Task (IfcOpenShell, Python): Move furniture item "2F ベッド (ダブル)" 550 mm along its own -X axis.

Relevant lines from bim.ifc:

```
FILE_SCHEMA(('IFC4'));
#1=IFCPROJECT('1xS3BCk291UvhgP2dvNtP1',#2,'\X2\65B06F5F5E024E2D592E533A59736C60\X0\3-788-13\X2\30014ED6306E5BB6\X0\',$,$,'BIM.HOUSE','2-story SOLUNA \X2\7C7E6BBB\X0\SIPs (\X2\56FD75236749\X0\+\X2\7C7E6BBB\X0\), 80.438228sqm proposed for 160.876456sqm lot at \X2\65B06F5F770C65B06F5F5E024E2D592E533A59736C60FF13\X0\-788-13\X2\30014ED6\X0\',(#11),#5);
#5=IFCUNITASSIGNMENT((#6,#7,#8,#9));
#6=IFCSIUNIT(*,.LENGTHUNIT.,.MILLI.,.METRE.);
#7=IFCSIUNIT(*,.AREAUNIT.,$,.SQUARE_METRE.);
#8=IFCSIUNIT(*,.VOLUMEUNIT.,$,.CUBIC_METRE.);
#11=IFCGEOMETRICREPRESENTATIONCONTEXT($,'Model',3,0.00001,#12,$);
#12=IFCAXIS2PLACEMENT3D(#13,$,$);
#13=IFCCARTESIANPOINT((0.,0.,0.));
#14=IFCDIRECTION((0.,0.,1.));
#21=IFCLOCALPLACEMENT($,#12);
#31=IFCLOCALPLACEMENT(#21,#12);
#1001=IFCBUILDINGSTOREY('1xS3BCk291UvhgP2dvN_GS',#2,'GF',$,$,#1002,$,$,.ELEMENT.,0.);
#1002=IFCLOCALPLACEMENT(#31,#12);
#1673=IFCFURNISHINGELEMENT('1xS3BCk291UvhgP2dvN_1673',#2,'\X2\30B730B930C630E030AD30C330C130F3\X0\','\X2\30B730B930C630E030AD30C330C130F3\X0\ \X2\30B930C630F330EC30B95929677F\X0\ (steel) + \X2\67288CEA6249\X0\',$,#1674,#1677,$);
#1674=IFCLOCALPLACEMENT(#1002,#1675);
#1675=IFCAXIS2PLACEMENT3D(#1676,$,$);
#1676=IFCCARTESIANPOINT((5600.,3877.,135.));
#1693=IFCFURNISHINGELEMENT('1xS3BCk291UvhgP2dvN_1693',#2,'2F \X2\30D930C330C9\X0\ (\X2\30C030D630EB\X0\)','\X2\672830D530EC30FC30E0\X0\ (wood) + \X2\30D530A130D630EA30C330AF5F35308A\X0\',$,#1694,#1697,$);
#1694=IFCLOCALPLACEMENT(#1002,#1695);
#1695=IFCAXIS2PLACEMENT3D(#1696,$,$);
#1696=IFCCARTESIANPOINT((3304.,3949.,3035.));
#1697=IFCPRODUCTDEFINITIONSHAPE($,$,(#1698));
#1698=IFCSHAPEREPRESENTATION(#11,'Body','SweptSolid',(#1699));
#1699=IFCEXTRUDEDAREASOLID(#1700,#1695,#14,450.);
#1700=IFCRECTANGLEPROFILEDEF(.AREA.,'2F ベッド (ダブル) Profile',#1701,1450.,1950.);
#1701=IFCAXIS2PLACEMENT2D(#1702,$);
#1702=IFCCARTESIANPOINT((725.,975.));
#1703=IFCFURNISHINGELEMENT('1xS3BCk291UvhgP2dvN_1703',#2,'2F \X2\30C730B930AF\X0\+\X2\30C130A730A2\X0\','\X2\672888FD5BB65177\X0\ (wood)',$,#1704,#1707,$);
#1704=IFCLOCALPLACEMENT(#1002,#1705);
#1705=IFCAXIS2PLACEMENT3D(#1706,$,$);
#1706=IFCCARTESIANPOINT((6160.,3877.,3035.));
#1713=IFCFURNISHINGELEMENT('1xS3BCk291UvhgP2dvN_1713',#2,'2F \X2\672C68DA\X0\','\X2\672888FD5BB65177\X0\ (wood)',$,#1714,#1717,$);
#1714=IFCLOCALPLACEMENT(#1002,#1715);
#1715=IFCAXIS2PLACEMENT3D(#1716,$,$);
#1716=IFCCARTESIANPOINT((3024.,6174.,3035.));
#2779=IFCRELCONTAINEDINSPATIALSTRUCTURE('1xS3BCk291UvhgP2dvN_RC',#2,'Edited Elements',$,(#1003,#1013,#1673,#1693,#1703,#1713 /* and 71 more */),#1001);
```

```python
import ifcopenshell
import ifcopenshell.api.geometry
import ifcopenshell.util.placement

model = ifcopenshell.open("bim.ifc")

item = model.by_guid("1xS3BCk291UvhgP2dvN_1693")
matrix = ifcopenshell.util.placement.get_local_placement(item.ObjectPlacement)
matrix[:3, 3] -= matrix[:3, 0] * 550.0
ifcopenshell.api.geometry.edit_object_placement(model, product=item, matrix=matrix, is_si=False)

print(ifcopenshell.util.placement.get_local_placement(item.ObjectPlacement).round(3) + 0.0)

model.write("bim_edited.ifc")
```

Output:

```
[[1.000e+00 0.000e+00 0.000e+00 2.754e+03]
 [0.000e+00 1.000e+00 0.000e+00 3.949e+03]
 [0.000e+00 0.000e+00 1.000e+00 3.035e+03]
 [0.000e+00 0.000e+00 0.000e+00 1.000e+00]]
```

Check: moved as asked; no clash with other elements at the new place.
